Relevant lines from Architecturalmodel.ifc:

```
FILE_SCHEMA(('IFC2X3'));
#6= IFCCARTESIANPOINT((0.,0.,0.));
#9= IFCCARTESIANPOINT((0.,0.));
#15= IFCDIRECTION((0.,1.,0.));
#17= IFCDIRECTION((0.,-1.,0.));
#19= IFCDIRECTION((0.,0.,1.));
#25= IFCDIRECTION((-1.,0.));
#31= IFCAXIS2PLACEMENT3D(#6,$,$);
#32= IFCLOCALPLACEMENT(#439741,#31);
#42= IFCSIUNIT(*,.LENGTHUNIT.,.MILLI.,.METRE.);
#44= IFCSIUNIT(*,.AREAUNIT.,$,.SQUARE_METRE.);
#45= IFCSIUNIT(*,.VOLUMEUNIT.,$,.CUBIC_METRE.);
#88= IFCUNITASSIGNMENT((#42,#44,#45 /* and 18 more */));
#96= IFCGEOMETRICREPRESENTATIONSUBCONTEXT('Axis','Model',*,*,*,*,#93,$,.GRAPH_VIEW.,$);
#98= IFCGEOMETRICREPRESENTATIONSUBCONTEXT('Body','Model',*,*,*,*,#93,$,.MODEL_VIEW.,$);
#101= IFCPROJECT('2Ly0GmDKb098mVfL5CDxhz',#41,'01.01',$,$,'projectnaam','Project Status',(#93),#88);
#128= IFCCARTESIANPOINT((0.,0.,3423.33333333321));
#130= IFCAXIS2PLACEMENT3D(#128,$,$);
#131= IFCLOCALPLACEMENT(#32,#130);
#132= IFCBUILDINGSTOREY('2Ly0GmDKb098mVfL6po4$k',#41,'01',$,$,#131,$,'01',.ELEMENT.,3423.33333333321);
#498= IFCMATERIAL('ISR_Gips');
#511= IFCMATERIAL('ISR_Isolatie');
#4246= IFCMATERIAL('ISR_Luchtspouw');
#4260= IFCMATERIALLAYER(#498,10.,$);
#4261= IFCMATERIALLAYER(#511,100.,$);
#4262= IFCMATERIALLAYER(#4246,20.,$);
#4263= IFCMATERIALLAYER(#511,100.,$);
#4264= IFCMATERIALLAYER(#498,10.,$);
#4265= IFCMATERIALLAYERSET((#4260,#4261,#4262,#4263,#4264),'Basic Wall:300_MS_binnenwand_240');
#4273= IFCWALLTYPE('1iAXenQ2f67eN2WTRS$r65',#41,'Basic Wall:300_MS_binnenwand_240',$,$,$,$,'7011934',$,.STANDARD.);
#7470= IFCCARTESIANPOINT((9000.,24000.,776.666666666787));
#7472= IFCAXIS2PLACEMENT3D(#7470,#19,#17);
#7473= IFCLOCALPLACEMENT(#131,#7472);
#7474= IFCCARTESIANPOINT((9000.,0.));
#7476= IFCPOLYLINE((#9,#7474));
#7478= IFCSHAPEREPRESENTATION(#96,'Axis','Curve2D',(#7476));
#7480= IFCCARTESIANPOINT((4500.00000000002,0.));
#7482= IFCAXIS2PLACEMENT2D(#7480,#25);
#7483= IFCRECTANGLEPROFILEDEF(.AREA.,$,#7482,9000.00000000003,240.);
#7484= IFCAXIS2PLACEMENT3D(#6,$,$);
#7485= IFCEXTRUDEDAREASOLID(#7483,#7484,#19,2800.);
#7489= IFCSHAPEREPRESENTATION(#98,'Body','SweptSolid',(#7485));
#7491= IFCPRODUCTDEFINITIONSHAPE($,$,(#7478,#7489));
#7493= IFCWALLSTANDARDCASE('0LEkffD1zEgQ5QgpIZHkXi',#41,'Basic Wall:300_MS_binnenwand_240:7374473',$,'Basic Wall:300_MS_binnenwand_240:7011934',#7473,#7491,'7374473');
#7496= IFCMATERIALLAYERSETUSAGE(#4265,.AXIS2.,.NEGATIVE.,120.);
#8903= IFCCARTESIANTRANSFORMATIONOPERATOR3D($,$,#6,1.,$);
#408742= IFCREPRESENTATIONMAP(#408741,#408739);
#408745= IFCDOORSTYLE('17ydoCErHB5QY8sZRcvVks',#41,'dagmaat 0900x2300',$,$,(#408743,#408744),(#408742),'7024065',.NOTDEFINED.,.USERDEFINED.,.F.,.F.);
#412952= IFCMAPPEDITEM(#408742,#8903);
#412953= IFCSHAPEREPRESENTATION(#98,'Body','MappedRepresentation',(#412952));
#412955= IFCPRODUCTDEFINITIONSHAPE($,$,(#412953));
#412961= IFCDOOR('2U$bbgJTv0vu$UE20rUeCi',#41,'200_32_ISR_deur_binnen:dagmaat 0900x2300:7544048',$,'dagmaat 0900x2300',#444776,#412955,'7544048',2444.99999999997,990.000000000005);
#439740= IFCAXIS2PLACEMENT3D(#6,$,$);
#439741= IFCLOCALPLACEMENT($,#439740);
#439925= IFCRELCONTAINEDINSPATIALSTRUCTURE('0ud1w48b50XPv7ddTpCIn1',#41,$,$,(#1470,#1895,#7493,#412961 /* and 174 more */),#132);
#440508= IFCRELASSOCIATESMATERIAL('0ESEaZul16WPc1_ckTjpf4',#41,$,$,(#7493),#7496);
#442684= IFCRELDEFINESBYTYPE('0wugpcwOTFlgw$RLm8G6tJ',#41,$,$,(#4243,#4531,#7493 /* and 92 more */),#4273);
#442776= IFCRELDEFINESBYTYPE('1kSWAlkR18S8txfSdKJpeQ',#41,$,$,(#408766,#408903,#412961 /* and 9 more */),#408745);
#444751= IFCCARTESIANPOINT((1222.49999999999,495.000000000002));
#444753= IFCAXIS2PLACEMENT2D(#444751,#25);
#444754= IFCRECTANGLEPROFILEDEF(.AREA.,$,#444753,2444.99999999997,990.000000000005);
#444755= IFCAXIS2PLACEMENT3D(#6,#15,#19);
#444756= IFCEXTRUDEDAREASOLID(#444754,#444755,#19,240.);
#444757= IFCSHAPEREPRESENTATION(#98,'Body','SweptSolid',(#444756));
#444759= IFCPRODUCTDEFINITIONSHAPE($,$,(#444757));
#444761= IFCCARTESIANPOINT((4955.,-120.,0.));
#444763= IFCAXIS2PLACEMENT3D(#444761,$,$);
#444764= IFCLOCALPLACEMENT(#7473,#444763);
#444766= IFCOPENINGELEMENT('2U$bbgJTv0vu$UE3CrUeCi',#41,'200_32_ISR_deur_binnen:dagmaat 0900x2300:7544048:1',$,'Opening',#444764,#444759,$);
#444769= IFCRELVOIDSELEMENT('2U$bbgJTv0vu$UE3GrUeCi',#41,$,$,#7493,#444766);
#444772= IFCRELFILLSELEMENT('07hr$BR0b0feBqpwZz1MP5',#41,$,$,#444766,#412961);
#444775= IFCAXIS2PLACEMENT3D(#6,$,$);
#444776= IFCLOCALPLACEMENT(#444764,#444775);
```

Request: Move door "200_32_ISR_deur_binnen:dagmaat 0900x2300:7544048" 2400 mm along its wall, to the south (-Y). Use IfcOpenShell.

```python
import ifcopenshell
import ifcopenshell.api.geometry
import ifcopenshell.util.placement

model = ifcopenshell.open("Architecturalmodel.ifc")

door = model.by_id(412961)
opening = door.FillsVoids[0].RelatingOpeningElement
wall = opening.VoidsElements[0].RelatingBuildingElement

wall_matrix = ifcopenshell.util.placement.get_local_placement(wall.ObjectPlacement)
shift = wall_matrix[:3, 0] * 2400.0
before = ifcopenshell.util.placement.get_local_placement(door.ObjectPlacement)[:3, 3].copy()

# The door is placed relative to its opening, so it follows when the opening moves.
matrix = ifcopenshell.util.placement.get_local_placement(opening.ObjectPlacement)
matrix[:3, 3] += shift
ifcopenshell.api.geometry.edit_object_placement(
    model, product=opening, matrix=matrix, is_si=False, should_transform_children=True
)

after = ifcopenshell.util.placement.get_local_placement(door.ObjectPlacement)[:3, 3]
print("door moved by", (after - before).round(3) + 0.0)

model.write("Architecturalmodel_rev.ifc")
```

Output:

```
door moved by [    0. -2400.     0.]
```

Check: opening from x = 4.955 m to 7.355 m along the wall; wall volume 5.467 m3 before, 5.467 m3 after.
